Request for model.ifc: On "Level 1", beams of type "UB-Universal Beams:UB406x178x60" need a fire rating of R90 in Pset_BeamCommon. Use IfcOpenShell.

First a look at what the model holds.

```python
import ifcopenshell
import ifcopenshell.util.element

model = ifcopenshell.open("model.ifc")
print(model.schema)
storey = next(s for s in model.by_type("IfcBuildingStorey") if s.Name == "Level 1")
beams = [e for e in ifcopenshell.util.element.get_decomposition(storey) if e.is_a("IfcBeam")]
seen = {}
for e in beams:
    element_type = ifcopenshell.util.element.get_type(e)
    key = (element_type.Name if element_type != e and element_type else None, ifcopenshell.util.element.get_pset(e, "Pset_BeamCommon", "FireRating"))
    seen[key] = seen.get(key, 0) + 1
for (name, value), count in sorted(seen.items(), key=str):
    print(count, "x", name, "|", value)
```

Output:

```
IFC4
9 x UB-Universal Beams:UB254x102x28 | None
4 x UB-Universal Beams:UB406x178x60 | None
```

```python
import ifcopenshell
import ifcopenshell.api.pset
import ifcopenshell.util.element

model = ifcopenshell.open("model.ifc")

storey = next(s for s in model.by_type("IfcBuildingStorey") if s.Name == "Level 1")
beams = [e for e in ifcopenshell.util.element.get_decomposition(storey) if e.is_a("IfcBeam")]

count = 0
for e in beams:
    element_type = ifcopenshell.util.element.get_type(e)
    if element_type in (None, e) or element_type.Name != "UB-Universal Beams:UB406x178x60":
        continue
    # add_pset returns the element's existing set when there is one.
    pset = ifcopenshell.api.pset.add_pset(model, product=e, name="Pset_BeamCommon")
    ifcopenshell.api.pset.edit_pset(model, pset=pset, properties={"FireRating": "R90"})
    count += 1

print(count, "beams updated")

model.write("model_edited.ifc")
```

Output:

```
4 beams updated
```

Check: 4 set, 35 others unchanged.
